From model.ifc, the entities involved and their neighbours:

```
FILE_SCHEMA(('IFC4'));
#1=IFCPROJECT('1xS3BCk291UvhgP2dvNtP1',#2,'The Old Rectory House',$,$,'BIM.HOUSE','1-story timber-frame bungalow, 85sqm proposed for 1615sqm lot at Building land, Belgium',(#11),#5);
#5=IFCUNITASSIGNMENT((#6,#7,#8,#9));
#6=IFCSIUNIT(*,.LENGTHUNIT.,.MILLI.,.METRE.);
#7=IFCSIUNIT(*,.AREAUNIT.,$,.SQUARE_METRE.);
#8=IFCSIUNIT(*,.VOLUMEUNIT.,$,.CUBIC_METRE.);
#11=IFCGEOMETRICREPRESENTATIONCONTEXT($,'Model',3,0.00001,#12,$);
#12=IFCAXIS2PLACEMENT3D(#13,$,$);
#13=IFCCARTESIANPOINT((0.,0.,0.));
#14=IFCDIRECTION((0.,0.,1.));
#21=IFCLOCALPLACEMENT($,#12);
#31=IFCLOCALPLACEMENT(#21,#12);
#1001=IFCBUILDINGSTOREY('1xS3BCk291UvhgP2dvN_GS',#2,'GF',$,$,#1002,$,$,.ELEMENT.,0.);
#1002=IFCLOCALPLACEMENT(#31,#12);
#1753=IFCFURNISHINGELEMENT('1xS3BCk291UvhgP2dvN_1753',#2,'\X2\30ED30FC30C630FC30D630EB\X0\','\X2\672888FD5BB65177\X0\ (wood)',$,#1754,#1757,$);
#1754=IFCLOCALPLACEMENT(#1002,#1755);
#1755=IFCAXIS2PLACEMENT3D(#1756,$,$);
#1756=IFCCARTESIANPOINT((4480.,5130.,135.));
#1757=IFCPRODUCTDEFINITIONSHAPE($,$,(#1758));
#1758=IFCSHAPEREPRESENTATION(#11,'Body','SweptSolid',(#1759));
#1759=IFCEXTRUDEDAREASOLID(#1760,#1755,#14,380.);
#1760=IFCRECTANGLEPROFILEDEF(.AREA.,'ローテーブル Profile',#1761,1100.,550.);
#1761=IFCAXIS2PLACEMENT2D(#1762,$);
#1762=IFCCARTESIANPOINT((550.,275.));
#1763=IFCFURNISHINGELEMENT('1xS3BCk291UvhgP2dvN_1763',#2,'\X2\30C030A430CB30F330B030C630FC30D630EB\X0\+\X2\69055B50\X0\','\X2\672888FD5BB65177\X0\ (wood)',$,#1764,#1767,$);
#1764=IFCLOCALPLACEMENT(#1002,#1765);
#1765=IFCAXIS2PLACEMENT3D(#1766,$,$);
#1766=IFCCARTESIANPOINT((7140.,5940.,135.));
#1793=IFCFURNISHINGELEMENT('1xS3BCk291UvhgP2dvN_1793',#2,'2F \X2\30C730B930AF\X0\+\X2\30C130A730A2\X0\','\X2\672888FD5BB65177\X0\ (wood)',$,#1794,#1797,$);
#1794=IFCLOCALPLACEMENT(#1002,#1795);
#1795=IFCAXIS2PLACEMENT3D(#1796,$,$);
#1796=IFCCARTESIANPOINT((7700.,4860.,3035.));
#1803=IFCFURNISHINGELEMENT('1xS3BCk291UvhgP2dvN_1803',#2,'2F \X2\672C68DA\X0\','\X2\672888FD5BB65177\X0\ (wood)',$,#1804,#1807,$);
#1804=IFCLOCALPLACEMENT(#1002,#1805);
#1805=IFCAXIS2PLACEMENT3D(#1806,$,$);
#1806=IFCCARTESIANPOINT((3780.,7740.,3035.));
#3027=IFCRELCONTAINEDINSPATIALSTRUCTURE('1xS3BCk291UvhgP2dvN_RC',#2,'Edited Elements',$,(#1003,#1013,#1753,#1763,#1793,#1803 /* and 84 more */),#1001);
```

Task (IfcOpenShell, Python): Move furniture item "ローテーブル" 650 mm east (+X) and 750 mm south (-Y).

```python
import ifcopenshell
import ifcopenshell.api.geometry
import ifcopenshell.util.placement

model = ifcopenshell.open("model.ifc")

item = model.by_guid("1xS3BCk291UvhgP2dvN_1753")
matrix = ifcopenshell.util.placement.get_local_placement(item.ObjectPlacement)
matrix[0, 3] += 650.0
matrix[1, 3] -= 750.0
ifcopenshell.api.geometry.edit_object_placement(model, product=item, matrix=matrix, is_si=False)

print(ifcopenshell.util.placement.get_local_placement(item.ObjectPlacement).round(3) + 0.0)

model.write("model_edited.ifc")
```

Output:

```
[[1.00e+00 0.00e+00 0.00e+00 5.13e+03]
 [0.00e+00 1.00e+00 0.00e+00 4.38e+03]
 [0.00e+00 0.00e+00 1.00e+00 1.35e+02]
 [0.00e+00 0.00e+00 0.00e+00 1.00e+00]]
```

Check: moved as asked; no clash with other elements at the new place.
